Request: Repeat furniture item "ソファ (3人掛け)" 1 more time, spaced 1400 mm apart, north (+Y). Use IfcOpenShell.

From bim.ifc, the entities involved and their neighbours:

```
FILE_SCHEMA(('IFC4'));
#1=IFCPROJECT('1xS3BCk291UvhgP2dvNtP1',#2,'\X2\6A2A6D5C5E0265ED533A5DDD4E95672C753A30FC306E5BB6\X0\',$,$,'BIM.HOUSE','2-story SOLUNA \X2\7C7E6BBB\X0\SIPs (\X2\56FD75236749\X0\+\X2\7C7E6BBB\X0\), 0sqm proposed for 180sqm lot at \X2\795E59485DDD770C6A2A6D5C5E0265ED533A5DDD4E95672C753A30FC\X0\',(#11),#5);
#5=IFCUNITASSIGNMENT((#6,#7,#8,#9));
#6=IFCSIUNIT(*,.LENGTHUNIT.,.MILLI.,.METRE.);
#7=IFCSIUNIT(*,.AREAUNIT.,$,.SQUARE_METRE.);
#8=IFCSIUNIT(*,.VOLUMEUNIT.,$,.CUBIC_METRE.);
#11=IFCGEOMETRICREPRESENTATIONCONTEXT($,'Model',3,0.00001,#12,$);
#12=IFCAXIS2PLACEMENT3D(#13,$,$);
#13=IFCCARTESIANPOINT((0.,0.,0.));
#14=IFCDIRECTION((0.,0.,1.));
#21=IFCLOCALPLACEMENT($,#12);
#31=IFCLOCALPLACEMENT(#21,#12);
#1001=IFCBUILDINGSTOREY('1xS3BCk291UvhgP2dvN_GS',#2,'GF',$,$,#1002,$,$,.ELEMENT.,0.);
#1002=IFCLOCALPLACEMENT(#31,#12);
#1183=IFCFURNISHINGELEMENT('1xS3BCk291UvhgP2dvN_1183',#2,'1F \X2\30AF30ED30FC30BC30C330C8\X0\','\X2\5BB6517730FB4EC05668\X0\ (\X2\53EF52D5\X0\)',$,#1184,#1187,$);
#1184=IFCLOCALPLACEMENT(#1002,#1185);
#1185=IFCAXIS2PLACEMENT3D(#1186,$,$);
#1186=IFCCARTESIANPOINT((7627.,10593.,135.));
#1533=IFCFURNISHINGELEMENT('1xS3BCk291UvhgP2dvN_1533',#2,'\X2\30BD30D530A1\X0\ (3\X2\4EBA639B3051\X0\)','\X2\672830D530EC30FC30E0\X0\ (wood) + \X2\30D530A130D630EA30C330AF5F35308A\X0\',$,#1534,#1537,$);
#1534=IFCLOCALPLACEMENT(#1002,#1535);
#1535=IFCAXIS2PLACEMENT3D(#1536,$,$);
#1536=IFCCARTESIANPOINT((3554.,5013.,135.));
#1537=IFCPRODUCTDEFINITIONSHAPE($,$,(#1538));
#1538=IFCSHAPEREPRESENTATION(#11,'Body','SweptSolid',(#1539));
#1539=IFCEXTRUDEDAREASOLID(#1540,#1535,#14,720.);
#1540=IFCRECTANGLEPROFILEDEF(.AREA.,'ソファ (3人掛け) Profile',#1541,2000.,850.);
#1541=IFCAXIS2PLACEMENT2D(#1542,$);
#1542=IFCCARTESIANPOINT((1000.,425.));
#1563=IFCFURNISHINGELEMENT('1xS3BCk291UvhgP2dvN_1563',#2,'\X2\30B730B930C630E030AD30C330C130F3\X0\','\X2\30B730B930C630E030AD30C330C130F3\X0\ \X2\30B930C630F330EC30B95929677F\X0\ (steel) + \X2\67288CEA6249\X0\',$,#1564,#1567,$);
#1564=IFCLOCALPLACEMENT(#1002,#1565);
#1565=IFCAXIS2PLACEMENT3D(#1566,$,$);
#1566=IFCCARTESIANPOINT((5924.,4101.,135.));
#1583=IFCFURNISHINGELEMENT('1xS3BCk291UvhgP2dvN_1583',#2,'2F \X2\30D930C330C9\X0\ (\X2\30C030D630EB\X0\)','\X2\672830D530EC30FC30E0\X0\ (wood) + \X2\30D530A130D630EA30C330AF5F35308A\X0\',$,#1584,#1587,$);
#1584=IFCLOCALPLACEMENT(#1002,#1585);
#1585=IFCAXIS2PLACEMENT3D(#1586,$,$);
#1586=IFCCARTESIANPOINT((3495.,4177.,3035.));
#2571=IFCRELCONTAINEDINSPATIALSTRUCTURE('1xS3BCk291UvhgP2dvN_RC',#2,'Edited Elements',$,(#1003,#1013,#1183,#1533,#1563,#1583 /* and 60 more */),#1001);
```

```python
import numpy as np
import ifcopenshell
import ifcopenshell.api.geometry
import ifcopenshell.api.root
import ifcopenshell.util.element
import ifcopenshell.util.placement

model = ifcopenshell.open("bim.ifc")


def reuse_history(source, copy):
    """copy_class also copies each property set's owner history, people and application; keep the originals."""
    for rel in copy.IsDefinedBy:
        if rel.is_a("IfcRelDefinesByProperties") and (history := rel.RelatingPropertyDefinition.OwnerHistory):
            rel.RelatingPropertyDefinition.OwnerHistory = source.OwnerHistory
            ifcopenshell.util.element.remove_deep2(model, history)


source = model.by_guid("1xS3BCk291UvhgP2dvN_1533")
base = ifcopenshell.util.placement.get_local_placement(source.ObjectPlacement)
step = np.array([0.0, 1.0, 0.0]) * 1400.0

for i in range(1, 2):
    copy = ifcopenshell.api.root.copy_class(model, product=source)
    copy.Representation = ifcopenshell.util.element.copy_deep(
        model, source.Representation, exclude=["IfcGeometricRepresentationContext", "IfcRepresentationMap"]
    )
    reuse_history(source, copy)
    matrix = base.copy()
    matrix[:3, 3] += i * step
    print("added at", matrix[:3, 3].round(3) + 0.0)
    ifcopenshell.api.geometry.edit_object_placement(model, product=copy, matrix=matrix, is_si=False)

model.write("bim_v2.ifc")
```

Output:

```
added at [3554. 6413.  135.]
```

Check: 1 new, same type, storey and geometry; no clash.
